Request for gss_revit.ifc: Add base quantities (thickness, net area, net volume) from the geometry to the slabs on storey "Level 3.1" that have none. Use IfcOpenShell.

First a look at what the model holds.

```python
import ifcopenshell
import ifcopenshell.util.element
import ifcopenshell.util.unit

model = ifcopenshell.open("gss_revit.ifc")
print(model.schema)
for unit_type in ("LENGTHUNIT", "AREAUNIT", "VOLUMEUNIT"):
    print(unit_type, ifcopenshell.util.unit.calculate_unit_scale(model, unit_type))
storey = next(s for s in model.by_type("IfcBuildingStorey") if s.Name == "Level 3.1")
slabs = [e for e in ifcopenshell.util.element.get_decomposition(storey) if e.is_a("IfcSlab")]
for e in sorted(slabs, key=lambda e: e.id()):
    print(e.id(), e.is_a(), e.Name, list(ifcopenshell.util.element.get_psets(e, qtos_only=True)), sep=" | ")
```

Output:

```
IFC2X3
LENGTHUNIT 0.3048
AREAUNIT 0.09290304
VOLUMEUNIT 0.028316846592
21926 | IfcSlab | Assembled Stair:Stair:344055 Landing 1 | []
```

```python
import ifcopenshell
import ifcopenshell.api.pset
import ifcopenshell.geom
import ifcopenshell.util.element
import ifcopenshell.util.shape
import ifcopenshell.util.unit

model = ifcopenshell.open("gss_revit.ifc")
unit_scale = ifcopenshell.util.unit.calculate_unit_scale(model)
area_scale = ifcopenshell.util.unit.calculate_unit_scale(model, "AREAUNIT")
volume_scale = ifcopenshell.util.unit.calculate_unit_scale(model, "VOLUMEUNIT")
settings = ifcopenshell.geom.settings()

storey = next(s for s in model.by_type("IfcBuildingStorey") if s.Name == "Level 3.1")
slabs = [e for e in ifcopenshell.util.element.get_decomposition(storey) if e.is_a("IfcSlab")]

for e in sorted(slabs, key=lambda e: e.id()):
    if ifcopenshell.util.element.get_psets(e, qtos_only=True, should_inherit=False):
        continue
    # Geometry comes back in metres, in the element's own axes.
    shape = ifcopenshell.geom.create_shape(settings, e)
    values = {
        "Width": ifcopenshell.util.shape.get_z(shape.geometry) / unit_scale,
        "NetArea": ifcopenshell.util.shape.get_footprint_area(shape.geometry) / area_scale,
        "NetVolume": ifcopenshell.util.shape.get_volume(shape.geometry) / volume_scale,
    }
    qto = ifcopenshell.api.pset.add_qto(model, product=e, name="BaseQuantities")
    ifcopenshell.api.pset.edit_qto(model, qto=qto, properties=values)
    print(e.id(), {k: round(v, 3) for k, v in values.items()})

model.write("gss_revit-out.ifc")
```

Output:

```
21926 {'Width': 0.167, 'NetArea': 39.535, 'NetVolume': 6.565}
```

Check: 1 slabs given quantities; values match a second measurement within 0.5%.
